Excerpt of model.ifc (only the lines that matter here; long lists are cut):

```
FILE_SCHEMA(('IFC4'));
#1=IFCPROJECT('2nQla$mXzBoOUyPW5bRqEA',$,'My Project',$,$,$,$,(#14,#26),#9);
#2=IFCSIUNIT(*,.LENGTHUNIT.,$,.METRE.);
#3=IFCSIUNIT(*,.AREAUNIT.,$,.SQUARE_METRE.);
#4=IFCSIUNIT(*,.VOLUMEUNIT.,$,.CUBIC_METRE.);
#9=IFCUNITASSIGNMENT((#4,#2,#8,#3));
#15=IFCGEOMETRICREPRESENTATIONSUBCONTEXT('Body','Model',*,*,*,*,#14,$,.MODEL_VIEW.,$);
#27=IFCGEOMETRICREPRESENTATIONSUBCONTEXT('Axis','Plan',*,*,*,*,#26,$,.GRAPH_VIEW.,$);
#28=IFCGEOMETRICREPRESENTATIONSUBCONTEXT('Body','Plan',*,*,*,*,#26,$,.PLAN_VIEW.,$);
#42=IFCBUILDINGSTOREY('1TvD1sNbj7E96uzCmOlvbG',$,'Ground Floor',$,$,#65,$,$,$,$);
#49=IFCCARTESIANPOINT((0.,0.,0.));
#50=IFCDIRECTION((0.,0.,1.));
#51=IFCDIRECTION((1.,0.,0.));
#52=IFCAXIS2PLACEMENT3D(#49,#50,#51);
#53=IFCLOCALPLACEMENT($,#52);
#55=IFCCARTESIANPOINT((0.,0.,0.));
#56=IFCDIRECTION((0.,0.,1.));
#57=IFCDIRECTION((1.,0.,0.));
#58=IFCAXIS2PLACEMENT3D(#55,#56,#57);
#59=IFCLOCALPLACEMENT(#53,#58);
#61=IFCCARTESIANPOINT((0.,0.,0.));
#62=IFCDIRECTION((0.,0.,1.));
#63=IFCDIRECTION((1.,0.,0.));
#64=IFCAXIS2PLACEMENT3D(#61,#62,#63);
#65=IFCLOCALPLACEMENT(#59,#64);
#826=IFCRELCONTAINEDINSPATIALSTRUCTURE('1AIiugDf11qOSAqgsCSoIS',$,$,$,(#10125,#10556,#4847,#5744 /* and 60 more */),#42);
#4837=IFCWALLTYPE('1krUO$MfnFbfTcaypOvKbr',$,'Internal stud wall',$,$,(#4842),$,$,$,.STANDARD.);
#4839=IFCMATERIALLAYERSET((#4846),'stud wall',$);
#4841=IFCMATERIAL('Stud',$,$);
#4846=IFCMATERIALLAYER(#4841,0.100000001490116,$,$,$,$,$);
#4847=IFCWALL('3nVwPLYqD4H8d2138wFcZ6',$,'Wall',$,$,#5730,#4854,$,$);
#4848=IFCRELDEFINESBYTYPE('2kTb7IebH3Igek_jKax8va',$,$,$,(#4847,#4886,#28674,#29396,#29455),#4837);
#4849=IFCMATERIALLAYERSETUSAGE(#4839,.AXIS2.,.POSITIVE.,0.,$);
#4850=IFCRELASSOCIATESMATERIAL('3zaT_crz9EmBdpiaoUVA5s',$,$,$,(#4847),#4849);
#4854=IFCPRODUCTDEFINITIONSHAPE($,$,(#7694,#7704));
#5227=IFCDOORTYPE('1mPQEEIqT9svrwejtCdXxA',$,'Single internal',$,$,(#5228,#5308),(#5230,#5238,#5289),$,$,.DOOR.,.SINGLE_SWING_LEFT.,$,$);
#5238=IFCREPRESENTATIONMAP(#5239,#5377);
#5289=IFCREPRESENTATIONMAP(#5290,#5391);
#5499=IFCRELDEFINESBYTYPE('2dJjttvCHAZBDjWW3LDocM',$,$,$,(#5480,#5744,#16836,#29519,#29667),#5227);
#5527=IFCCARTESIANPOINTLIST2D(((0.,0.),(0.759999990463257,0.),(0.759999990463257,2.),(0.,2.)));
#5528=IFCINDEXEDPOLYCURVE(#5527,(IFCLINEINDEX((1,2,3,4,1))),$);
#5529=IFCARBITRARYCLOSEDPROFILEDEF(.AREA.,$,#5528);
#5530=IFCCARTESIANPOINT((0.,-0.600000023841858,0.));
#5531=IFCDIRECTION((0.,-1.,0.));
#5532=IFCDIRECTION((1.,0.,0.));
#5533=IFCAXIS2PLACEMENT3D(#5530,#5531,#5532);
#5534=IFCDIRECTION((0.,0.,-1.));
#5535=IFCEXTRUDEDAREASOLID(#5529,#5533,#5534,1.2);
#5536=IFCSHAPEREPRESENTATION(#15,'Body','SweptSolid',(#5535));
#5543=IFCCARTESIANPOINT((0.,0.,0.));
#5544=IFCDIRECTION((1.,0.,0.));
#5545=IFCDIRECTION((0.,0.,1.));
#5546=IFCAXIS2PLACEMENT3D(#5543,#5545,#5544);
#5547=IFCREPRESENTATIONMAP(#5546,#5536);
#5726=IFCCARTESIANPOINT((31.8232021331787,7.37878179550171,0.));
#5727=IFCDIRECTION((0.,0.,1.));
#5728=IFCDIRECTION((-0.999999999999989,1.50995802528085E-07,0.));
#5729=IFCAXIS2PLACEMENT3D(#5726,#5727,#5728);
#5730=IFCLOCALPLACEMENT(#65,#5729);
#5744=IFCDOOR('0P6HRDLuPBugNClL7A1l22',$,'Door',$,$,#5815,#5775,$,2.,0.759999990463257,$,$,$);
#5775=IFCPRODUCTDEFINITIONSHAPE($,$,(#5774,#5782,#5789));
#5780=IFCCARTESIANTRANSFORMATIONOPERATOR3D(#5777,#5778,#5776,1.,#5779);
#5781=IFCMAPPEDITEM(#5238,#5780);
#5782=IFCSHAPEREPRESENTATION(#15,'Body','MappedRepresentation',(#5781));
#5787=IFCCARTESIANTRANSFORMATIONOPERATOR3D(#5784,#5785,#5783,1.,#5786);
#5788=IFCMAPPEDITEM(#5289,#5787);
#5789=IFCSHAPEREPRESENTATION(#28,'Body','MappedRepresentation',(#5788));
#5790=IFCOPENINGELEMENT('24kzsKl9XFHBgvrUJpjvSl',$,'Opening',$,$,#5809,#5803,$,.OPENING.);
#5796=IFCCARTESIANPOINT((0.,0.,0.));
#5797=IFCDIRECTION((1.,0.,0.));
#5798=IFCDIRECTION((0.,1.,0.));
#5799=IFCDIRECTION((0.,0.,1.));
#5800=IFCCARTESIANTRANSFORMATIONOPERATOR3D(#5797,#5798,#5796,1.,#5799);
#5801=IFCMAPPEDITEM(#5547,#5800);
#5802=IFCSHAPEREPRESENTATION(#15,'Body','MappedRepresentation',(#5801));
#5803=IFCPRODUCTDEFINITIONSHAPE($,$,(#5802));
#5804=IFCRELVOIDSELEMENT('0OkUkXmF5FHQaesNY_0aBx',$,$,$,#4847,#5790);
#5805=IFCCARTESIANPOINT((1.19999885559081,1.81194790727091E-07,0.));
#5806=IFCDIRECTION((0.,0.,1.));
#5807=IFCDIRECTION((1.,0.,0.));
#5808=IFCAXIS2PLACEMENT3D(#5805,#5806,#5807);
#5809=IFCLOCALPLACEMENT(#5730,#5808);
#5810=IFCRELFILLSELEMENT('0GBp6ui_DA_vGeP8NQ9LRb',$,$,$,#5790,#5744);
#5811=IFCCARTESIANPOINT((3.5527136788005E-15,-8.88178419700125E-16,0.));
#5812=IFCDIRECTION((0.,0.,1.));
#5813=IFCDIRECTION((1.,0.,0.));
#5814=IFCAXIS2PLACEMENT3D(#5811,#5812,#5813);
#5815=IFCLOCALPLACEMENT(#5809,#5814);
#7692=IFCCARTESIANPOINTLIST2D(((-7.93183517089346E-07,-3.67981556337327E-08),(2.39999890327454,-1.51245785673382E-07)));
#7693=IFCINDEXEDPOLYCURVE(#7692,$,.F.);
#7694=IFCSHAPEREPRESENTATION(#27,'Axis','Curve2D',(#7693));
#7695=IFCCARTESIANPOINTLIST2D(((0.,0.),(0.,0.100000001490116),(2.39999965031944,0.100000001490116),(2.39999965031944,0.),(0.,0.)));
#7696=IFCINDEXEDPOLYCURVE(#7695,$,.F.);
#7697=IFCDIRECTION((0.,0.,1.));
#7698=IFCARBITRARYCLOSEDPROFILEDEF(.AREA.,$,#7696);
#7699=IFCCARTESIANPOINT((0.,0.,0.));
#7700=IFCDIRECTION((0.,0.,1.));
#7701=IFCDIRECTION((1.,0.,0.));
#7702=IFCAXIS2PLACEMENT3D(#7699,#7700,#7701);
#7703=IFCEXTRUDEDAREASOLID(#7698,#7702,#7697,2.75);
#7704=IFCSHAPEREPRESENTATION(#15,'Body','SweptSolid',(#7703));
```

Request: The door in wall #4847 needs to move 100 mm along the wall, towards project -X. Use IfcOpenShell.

```python
import ifcopenshell
import ifcopenshell.api.geometry
import ifcopenshell.util.placement

model = ifcopenshell.open("model.ifc")

door = model.by_guid("0P6HRDLuPBugNClL7A1l22")
opening = door.FillsVoids[0].RelatingOpeningElement
wall = opening.VoidsElements[0].RelatingBuildingElement

wall_matrix = ifcopenshell.util.placement.get_local_placement(wall.ObjectPlacement)
shift = wall_matrix[:3, 0] * 0.1
before = ifcopenshell.util.placement.get_local_placement(door.ObjectPlacement)[:3, 3].copy()

# The door is placed relative to its opening, so it follows when the opening moves.
matrix = ifcopenshell.util.placement.get_local_placement(opening.ObjectPlacement)
matrix[:3, 3] += shift
ifcopenshell.api.geometry.edit_object_placement(
    model, product=opening, matrix=matrix, is_si=False, should_transform_children=True
)

after = ifcopenshell.util.placement.get_local_placement(door.ObjectPlacement)[:3, 3]
print("door moved by", (after - before).round(3) + 0.0)

model.write("model_rev.ifc")
```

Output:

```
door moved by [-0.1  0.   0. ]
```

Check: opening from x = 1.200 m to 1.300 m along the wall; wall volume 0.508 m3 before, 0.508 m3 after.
